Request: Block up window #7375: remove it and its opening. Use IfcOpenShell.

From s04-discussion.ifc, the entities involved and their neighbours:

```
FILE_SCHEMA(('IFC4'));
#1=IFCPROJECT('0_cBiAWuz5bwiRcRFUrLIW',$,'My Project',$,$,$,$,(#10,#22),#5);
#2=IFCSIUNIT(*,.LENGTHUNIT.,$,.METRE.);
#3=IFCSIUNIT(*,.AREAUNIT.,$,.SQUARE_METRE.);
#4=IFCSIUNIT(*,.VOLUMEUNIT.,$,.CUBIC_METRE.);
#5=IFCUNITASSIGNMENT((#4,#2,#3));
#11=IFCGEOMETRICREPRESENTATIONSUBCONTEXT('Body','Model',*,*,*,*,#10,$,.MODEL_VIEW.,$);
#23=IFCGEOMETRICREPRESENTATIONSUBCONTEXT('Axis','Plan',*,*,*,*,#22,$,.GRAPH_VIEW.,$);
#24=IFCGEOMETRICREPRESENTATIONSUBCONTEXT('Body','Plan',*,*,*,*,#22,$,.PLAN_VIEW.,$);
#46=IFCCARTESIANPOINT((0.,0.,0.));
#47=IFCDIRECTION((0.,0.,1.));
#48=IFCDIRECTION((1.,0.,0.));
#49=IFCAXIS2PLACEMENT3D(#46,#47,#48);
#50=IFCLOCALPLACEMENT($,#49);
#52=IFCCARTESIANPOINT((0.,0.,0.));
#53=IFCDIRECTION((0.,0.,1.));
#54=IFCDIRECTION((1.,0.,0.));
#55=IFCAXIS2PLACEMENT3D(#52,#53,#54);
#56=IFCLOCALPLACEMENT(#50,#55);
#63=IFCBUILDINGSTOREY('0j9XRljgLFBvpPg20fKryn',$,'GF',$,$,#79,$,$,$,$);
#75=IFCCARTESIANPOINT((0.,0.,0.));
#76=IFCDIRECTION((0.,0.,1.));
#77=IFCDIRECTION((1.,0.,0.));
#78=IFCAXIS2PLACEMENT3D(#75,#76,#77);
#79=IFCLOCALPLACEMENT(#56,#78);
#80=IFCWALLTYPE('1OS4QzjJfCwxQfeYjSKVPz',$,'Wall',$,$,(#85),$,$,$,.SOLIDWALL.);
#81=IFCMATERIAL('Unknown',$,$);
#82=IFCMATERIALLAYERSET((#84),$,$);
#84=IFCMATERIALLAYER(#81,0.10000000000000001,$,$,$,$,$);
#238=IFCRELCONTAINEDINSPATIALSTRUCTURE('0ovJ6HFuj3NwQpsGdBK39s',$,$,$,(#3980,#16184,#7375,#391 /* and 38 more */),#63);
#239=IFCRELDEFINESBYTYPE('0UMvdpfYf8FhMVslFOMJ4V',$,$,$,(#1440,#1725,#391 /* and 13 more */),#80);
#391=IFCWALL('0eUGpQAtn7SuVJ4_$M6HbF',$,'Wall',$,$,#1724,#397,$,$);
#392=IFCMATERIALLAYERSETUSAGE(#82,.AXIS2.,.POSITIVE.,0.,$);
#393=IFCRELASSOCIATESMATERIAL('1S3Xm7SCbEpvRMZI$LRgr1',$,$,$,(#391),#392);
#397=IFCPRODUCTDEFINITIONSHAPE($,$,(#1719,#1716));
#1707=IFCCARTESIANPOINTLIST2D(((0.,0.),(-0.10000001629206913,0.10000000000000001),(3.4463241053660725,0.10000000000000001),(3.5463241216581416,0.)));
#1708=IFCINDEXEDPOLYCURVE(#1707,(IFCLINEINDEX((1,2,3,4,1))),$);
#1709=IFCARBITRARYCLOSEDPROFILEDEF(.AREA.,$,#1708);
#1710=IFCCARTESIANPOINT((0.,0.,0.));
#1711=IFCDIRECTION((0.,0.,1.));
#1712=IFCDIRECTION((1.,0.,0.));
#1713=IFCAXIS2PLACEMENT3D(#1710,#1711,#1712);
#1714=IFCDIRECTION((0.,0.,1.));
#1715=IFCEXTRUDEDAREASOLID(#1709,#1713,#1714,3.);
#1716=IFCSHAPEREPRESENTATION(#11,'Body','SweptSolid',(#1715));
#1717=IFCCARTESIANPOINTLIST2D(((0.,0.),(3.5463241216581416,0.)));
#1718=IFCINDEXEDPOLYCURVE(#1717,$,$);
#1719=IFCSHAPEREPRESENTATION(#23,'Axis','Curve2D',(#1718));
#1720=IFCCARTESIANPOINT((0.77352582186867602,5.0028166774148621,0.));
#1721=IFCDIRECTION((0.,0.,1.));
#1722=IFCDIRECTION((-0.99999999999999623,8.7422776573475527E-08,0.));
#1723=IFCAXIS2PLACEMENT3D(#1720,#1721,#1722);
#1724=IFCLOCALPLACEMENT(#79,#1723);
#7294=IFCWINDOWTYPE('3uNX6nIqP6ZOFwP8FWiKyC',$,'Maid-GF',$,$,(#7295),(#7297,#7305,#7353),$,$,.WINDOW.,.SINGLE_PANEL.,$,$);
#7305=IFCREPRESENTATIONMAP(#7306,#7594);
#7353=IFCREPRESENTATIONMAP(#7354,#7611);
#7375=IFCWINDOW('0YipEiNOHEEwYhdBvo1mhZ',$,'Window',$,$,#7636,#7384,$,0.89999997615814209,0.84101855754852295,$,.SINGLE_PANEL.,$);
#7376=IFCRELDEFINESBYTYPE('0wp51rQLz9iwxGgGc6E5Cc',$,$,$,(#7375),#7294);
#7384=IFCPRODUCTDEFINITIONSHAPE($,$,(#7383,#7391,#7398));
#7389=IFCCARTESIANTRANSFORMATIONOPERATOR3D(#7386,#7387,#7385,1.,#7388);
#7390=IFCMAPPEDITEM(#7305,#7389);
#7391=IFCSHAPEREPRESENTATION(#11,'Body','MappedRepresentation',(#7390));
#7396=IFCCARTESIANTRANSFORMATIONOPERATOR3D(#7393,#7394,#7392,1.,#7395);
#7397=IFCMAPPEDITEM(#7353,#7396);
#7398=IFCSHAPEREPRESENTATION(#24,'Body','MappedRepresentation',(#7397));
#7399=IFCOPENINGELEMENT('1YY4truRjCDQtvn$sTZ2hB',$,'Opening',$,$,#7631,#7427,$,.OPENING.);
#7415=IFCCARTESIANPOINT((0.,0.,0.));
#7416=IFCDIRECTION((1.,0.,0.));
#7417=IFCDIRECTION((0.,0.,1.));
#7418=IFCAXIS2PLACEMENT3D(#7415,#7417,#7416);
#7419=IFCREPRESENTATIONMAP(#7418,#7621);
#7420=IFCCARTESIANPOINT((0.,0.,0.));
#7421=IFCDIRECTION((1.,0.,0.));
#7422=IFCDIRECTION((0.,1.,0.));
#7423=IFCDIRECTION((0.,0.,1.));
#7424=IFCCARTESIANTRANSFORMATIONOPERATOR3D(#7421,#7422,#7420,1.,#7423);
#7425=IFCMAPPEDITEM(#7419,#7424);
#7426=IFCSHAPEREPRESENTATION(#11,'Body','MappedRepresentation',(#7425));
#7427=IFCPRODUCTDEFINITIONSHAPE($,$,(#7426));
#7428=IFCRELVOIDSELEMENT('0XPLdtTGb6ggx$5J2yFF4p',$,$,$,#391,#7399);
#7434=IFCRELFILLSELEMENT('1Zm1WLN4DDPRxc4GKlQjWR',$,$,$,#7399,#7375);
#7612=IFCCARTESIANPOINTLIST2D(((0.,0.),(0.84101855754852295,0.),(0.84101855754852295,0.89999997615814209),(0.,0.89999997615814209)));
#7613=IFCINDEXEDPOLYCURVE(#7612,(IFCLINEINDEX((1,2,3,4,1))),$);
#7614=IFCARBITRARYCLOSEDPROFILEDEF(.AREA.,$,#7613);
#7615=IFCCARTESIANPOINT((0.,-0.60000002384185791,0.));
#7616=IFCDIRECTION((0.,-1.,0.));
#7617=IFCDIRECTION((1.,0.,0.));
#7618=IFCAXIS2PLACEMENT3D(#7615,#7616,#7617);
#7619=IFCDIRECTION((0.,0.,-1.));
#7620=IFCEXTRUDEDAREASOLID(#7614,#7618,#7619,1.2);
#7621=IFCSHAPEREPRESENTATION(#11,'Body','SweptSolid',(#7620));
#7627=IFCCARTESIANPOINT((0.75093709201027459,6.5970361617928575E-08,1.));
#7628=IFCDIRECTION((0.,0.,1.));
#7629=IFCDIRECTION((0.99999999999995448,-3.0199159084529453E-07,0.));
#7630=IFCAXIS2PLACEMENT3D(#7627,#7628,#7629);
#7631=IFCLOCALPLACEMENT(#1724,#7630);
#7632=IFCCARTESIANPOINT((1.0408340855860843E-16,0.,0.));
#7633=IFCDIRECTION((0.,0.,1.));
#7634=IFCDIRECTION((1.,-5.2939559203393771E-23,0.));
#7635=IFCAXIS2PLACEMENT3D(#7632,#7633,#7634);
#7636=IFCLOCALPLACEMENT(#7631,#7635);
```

```python
import ifcopenshell
import ifcopenshell.api.feature
import ifcopenshell.api.root
import ifcopenshell.geom
import ifcopenshell.util.shape

model = ifcopenshell.open("s04-discussion.ifc")
settings = ifcopenshell.geom.settings()


def volume(element):
    """Net volume in cubic metres, openings subtracted."""
    shape = ifcopenshell.geom.create_shape(settings, element)
    return ifcopenshell.util.shape.get_volume(shape.geometry)


window = model.by_guid("0YipEiNOHEEwYhdBvo1mhZ")
opening = window.FillsVoids[0].RelatingOpeningElement
wall = opening.VoidsElements[0].RelatingBuildingElement
before = volume(wall)

ifcopenshell.api.root.remove_product(model, product=window)
ifcopenshell.api.feature.remove_feature(model, feature=opening)

after = volume(wall)

print(f"wall volume {before:.3f} -> {after:.3f} m3")

model.write("s04-discussion_updated.ifc")
```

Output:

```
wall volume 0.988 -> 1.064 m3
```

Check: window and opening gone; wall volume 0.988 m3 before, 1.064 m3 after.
